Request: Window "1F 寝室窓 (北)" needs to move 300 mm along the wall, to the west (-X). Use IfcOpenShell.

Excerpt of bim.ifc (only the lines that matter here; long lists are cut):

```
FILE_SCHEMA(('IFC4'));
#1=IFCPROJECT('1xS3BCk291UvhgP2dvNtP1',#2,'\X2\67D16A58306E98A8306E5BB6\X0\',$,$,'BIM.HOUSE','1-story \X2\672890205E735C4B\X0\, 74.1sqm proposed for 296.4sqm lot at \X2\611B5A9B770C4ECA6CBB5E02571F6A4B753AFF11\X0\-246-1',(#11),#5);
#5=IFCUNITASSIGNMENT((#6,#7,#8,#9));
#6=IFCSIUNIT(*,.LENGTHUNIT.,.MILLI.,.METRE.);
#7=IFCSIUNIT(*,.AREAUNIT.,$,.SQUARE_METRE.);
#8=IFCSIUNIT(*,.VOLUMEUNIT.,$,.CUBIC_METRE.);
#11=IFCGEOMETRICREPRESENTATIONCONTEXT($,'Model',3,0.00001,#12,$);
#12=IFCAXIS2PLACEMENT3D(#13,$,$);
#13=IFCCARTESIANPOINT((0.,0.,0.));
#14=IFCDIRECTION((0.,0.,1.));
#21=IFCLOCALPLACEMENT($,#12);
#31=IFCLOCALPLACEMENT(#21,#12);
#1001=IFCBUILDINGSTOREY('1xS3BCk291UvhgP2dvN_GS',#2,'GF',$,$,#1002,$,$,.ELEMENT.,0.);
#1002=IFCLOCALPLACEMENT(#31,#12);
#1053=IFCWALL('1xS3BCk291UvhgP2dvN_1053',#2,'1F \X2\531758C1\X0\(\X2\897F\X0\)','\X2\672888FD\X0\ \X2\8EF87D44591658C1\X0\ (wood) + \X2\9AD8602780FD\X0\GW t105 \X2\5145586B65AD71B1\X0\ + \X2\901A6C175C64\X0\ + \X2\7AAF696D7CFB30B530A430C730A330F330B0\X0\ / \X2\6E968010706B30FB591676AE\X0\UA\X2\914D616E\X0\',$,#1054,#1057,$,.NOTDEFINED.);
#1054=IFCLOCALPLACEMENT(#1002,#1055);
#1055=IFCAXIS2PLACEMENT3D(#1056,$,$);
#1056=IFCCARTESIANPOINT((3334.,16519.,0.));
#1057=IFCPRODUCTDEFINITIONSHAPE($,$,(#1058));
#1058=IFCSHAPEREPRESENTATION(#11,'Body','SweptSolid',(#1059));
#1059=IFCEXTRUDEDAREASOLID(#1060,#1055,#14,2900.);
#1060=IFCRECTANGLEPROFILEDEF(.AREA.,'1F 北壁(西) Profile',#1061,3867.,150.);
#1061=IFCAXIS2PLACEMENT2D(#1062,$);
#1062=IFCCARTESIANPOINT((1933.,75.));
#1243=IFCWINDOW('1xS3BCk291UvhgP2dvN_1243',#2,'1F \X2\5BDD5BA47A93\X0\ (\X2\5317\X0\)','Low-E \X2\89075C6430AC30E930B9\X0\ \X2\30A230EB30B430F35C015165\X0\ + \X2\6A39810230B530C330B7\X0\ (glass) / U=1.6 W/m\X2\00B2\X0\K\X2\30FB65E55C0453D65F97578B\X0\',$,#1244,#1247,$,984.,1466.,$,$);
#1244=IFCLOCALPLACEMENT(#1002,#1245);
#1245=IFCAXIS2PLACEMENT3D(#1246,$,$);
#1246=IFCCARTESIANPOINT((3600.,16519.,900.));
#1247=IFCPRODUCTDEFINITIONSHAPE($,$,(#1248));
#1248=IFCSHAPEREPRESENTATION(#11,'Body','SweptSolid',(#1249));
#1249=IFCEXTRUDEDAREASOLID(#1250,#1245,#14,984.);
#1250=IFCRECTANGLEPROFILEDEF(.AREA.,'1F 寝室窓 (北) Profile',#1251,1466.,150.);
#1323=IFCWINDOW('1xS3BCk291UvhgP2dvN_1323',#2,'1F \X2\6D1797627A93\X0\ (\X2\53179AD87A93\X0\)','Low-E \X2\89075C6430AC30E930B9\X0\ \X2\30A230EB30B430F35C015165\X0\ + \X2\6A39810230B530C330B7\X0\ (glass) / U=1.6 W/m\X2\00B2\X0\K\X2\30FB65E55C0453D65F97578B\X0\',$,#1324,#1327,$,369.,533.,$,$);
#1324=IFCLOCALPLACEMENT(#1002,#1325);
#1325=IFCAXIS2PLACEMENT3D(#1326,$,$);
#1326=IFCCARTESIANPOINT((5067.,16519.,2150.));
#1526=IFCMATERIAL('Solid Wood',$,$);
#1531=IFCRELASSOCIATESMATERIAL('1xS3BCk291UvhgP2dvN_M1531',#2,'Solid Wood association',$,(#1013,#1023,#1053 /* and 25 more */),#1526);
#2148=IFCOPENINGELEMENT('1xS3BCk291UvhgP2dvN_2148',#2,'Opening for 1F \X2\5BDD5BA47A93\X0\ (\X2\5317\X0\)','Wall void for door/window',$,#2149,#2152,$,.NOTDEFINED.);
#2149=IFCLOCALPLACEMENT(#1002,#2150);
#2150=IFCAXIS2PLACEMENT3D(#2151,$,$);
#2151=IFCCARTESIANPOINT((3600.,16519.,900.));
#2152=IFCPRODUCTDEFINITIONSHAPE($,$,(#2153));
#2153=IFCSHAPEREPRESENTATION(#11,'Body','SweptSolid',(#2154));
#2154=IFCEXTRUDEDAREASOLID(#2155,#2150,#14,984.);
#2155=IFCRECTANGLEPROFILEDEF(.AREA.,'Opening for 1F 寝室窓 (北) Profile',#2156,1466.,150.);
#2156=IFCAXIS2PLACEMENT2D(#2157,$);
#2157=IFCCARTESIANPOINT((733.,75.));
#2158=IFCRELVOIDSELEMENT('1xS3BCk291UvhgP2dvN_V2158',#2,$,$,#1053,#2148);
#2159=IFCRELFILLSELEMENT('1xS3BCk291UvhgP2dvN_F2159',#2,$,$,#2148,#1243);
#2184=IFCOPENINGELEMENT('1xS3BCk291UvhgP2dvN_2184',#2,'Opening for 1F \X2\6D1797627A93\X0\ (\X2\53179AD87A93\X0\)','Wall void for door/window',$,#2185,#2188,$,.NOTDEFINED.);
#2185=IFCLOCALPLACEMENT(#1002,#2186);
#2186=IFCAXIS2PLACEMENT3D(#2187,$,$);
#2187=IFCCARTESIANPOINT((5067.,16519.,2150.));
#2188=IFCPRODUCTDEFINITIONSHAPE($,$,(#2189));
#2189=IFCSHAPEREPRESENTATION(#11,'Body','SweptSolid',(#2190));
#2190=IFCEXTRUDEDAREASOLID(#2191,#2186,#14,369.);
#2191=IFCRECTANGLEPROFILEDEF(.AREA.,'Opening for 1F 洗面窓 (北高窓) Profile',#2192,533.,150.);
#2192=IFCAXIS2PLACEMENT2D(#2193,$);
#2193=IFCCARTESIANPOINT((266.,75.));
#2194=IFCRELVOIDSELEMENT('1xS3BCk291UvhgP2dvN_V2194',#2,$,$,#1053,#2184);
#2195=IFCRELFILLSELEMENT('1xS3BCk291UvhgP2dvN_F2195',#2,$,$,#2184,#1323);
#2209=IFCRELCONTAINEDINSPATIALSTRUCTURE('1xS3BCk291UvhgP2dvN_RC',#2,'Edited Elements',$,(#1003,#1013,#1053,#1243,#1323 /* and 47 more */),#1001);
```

```python
import ifcopenshell
import ifcopenshell.api.geometry
import ifcopenshell.util.placement
import ifcopenshell.util.unit

model = ifcopenshell.open("bim.ifc")
unit_scale = ifcopenshell.util.unit.calculate_unit_scale(model)

window = model.by_id(1243)
opening = window.FillsVoids[0].RelatingOpeningElement
wall = opening.VoidsElements[0].RelatingBuildingElement

wall_matrix = ifcopenshell.util.placement.get_local_placement(wall.ObjectPlacement)
shift = wall_matrix[:3, 0] * -0.3 / unit_scale
before = ifcopenshell.util.placement.get_local_placement(window.ObjectPlacement)[:3, 3].copy()

# The window is not placed relative to its opening, so move both.
for product in (opening, window):
    matrix = ifcopenshell.util.placement.get_local_placement(product.ObjectPlacement)
    matrix[:3, 3] += shift
    ifcopenshell.api.geometry.edit_object_placement(model, product=product, matrix=matrix, is_si=False)

after = ifcopenshell.util.placement.get_local_placement(window.ObjectPlacement)[:3, 3]
print("window moved by", (after - before).round(3) + 0.0)

model.write("bim_rev.ifc")
```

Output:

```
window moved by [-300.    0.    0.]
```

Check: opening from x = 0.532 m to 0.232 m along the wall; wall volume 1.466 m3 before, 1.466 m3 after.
